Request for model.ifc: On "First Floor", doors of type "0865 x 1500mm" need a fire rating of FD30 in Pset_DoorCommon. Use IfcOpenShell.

First a look at what the model holds.

```python
import ifcopenshell
import ifcopenshell.util.element

model = ifcopenshell.open("model.ifc")
print(model.schema)
storey = next(s for s in model.by_type("IfcBuildingStorey") if s.Name == "First Floor")
doors = [e for e in ifcopenshell.util.element.get_decomposition(storey) if e.is_a("IfcDoor")]
seen = {}
for e in doors:
    element_type = ifcopenshell.util.element.get_type(e)
    key = (element_type.Name if element_type != e and element_type else None, ifcopenshell.util.element.get_pset(e, "Pset_DoorCommon", "FireRating"))
    seen[key] = seen.get(key, 0) + 1
for (name, value), count in sorted(seen.items(), key=str):
    print(count, "x", name, "|", value)
```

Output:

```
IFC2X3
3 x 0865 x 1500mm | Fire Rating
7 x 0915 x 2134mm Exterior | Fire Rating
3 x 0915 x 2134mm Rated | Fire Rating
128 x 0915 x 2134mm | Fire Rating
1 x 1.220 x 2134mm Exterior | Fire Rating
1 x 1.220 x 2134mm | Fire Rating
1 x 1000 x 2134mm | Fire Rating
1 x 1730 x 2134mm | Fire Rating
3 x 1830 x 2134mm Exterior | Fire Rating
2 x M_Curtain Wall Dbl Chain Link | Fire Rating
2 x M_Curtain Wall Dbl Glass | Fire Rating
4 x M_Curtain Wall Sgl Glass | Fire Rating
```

```python
import ifcopenshell
import ifcopenshell.api.pset
import ifcopenshell.util.element

model = ifcopenshell.open("model.ifc")

storey = next(s for s in model.by_type("IfcBuildingStorey") if s.Name == "First Floor")
doors = [e for e in ifcopenshell.util.element.get_decomposition(storey) if e.is_a("IfcDoor")]

count = 0
for e in doors:
    element_type = ifcopenshell.util.element.get_type(e)
    if element_type in (None, e) or element_type.Name != "0865 x 1500mm":
        continue
    # add_pset returns the element's existing set when there is one.
    pset = ifcopenshell.api.pset.add_pset(model, product=e, name="Pset_DoorCommon")
    ifcopenshell.api.pset.edit_pset(model, pset=pset, properties={"FireRating": "FD30"})
    count += 1

print(count, "doors updated")

model.write("model_rev.ifc")
```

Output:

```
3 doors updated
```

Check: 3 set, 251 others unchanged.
